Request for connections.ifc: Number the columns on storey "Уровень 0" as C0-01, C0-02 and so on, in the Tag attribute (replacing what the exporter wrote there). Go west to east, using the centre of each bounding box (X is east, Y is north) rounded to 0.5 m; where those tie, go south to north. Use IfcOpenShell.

First a look at what the model holds.

```python
import ifcopenshell
import ifcopenshell.util.element
import ifcopenshell.util.placement

model = ifcopenshell.open("connections.ifc")
print(model.schema)
storey = next(s for s in model.by_type("IfcBuildingStorey") if s.Name == "Уровень 0")
columns = [e for e in ifcopenshell.util.element.get_decomposition(storey) if e.is_a("IfcColumn")]
for e in sorted(columns, key=lambda e: e.id()):
    origin = ifcopenshell.util.placement.get_local_placement(e.ObjectPlacement)[:3, 3]
    print(e.id(), e.Tag, e.Name, origin.round(2) + 0.0, sep=" | ")
```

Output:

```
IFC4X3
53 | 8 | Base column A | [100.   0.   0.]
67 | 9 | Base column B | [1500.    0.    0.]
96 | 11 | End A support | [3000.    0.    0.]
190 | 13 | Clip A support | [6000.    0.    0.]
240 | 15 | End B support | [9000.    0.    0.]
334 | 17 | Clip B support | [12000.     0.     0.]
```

```python
import ifcopenshell
import ifcopenshell.geom
import ifcopenshell.util.element
import ifcopenshell.util.shape

model = ifcopenshell.open("connections.ifc")
settings = ifcopenshell.geom.settings()
settings.set("use-world-coords", True)


def centre(element):
    shape = ifcopenshell.geom.create_shape(settings, element)
    return ifcopenshell.util.shape.get_bbox_centroid(shape.geometry)


storey = next(s for s in model.by_type("IfcBuildingStorey") if s.Name == "Уровень 0")
columns = [e for e in ifcopenshell.util.element.get_decomposition(storey) if e.is_a("IfcColumn")]

# Insertion points can sit at a corner or the storey origin, so sort by the geometry (in metres).
centres = {e: centre(e) for e in columns}
columns.sort(key=lambda e: (round(centres[e][0] / 0.5), centres[e][1]))

for i, e in enumerate(columns, start=1):
    number = f"C0-{i:02d}"
    e.Tag = number
    print(e.id(), number)

model.write("connections_edited.ifc")
```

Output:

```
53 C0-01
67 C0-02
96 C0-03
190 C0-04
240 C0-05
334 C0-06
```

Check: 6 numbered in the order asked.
